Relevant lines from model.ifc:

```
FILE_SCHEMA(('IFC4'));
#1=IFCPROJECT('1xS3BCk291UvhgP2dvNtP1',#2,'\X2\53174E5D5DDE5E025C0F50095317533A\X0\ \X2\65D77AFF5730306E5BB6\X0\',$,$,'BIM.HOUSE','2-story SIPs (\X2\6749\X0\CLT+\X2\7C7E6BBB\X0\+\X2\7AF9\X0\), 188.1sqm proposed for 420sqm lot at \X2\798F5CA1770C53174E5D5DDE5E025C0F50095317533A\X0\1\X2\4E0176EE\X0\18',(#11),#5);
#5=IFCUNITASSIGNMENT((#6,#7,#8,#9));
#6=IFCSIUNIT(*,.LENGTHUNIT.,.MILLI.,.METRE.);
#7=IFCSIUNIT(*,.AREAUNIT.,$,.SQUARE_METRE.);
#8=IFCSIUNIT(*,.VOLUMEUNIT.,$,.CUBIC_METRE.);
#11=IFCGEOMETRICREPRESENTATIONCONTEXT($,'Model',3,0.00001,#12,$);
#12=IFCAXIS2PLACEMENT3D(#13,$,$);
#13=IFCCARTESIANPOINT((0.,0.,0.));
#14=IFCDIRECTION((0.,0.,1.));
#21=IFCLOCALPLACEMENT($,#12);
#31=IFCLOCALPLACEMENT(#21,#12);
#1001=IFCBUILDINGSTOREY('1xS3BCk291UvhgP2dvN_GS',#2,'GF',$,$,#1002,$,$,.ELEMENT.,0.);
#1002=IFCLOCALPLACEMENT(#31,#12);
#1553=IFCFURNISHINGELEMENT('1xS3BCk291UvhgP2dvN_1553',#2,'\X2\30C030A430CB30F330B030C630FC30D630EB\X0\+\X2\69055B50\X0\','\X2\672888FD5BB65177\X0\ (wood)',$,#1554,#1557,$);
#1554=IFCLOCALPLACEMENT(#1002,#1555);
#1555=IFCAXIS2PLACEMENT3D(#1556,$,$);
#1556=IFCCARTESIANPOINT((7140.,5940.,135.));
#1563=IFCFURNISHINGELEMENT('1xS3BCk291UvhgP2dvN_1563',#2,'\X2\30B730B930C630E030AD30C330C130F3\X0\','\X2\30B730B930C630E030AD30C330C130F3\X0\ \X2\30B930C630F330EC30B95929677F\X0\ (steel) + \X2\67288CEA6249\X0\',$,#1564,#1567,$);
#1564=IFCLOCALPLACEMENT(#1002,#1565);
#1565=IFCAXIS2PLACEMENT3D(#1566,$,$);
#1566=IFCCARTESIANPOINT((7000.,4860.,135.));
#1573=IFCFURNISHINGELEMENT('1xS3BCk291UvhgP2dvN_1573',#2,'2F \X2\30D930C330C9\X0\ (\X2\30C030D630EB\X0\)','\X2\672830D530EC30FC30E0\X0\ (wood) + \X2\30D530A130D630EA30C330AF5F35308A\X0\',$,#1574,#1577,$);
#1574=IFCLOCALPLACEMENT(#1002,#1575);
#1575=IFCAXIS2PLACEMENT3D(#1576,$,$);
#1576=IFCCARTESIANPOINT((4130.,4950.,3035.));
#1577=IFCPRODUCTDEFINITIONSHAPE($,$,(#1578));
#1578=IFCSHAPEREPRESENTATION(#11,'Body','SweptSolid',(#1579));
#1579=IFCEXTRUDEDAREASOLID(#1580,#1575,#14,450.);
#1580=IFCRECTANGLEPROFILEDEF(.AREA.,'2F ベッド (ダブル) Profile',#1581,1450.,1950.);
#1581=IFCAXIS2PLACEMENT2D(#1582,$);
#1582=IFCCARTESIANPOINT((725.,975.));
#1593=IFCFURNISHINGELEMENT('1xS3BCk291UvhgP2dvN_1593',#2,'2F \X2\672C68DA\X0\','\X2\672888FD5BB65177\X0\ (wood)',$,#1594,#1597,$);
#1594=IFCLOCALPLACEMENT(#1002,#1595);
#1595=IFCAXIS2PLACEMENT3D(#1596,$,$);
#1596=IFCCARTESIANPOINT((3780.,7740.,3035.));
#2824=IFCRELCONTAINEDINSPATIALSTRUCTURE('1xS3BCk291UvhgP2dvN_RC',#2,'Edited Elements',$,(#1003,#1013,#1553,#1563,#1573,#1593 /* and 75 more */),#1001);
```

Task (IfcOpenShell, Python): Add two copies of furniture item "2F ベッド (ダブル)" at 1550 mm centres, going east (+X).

```python
import numpy as np
import ifcopenshell
import ifcopenshell.api.geometry
import ifcopenshell.api.root
import ifcopenshell.util.element
import ifcopenshell.util.placement
import ifcopenshell.util.unit

model = ifcopenshell.open("model.ifc")
unit_scale = ifcopenshell.util.unit.calculate_unit_scale(model)


def reuse_history(source, copy):
    """copy_class also copies each property set's owner history, people and application; keep the originals."""
    for rel in copy.IsDefinedBy:
        if rel.is_a("IfcRelDefinesByProperties") and (history := rel.RelatingPropertyDefinition.OwnerHistory):
            rel.RelatingPropertyDefinition.OwnerHistory = source.OwnerHistory
            ifcopenshell.util.element.remove_deep2(model, history)


source = model.by_id(1573)
base = ifcopenshell.util.placement.get_local_placement(source.ObjectPlacement)
step = np.array([1.0, 0.0, 0.0]) * 1.55 / unit_scale

for i in range(1, 3):
    copy = ifcopenshell.api.root.copy_class(model, product=source)
    copy.Representation = ifcopenshell.util.element.copy_deep(
        model, source.Representation, exclude=["IfcGeometricRepresentationContext", "IfcRepresentationMap"]
    )
    reuse_history(source, copy)
    matrix = base.copy()
    matrix[:3, 3] += i * step
    print("added at", matrix[:3, 3].round(3) + 0.0)
    ifcopenshell.api.geometry.edit_object_placement(model, product=copy, matrix=matrix, is_si=False)

model.write("model-out.ifc")
```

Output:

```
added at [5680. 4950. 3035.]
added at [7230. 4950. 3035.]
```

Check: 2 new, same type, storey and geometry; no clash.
